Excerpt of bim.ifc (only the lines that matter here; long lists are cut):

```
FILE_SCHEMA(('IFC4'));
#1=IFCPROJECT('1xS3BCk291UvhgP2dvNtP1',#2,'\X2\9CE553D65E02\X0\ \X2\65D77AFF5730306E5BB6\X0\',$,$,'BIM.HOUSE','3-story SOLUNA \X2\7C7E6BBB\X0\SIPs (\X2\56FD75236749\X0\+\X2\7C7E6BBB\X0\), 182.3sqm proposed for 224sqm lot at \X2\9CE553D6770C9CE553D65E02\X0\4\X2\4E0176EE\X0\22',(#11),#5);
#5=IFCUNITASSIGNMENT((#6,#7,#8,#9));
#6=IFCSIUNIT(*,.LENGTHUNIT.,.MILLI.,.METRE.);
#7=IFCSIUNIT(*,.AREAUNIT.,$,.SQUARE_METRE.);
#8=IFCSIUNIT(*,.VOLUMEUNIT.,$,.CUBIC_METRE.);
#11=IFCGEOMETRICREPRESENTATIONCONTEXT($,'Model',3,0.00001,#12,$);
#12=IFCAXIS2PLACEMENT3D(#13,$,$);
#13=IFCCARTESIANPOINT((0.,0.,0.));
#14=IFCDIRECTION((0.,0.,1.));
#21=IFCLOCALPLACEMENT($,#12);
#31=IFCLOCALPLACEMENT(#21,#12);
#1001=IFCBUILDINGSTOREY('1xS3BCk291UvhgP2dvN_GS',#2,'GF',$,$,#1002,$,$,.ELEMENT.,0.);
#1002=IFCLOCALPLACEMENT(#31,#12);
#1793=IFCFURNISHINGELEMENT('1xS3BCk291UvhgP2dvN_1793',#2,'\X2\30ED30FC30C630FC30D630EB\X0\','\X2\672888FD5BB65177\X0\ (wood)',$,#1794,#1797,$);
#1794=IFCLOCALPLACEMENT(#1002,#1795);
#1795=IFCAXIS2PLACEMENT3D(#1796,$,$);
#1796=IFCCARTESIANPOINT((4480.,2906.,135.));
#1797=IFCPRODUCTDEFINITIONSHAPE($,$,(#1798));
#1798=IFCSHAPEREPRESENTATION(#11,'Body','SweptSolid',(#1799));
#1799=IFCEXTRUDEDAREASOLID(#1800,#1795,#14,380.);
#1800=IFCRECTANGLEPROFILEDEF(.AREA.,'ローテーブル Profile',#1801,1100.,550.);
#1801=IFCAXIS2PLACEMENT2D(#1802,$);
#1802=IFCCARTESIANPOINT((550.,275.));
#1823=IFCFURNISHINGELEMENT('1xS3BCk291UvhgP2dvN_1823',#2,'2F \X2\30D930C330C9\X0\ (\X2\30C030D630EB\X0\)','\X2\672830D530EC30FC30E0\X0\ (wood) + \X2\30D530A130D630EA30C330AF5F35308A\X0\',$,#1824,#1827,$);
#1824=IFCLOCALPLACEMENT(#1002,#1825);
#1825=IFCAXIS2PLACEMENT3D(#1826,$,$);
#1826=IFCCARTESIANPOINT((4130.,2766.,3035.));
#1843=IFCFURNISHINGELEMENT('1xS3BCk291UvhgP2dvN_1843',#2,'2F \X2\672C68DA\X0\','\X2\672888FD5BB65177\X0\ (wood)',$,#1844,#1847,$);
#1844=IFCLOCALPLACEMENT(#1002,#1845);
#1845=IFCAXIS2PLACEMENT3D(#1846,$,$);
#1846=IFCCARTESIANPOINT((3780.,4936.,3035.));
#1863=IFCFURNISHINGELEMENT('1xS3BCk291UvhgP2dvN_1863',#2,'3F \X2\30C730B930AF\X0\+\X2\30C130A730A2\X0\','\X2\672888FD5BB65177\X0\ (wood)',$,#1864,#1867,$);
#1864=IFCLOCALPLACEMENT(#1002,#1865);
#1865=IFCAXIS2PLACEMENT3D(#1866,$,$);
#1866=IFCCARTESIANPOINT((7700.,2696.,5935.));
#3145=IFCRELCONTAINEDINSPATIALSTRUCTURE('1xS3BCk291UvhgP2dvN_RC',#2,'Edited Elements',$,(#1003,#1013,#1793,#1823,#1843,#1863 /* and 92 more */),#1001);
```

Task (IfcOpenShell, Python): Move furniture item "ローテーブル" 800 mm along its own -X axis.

```python
import ifcopenshell
import ifcopenshell.api.geometry
import ifcopenshell.util.placement
import ifcopenshell.util.unit

model = ifcopenshell.open("bim.ifc")
unit_scale = ifcopenshell.util.unit.calculate_unit_scale(model)

item = model.by_guid("1xS3BCk291UvhgP2dvN_1793")
matrix = ifcopenshell.util.placement.get_local_placement(item.ObjectPlacement)
matrix[:3, 3] -= matrix[:3, 0] * 0.8 / unit_scale
ifcopenshell.api.geometry.edit_object_placement(model, product=item, matrix=matrix, is_si=False)

print(ifcopenshell.util.placement.get_local_placement(item.ObjectPlacement).round(3) + 0.0)

model.write("bim_rev.ifc")
```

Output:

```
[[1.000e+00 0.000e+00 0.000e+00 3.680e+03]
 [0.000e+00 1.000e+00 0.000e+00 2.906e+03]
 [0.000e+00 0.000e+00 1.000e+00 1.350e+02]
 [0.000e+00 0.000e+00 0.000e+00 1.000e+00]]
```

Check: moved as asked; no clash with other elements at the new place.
